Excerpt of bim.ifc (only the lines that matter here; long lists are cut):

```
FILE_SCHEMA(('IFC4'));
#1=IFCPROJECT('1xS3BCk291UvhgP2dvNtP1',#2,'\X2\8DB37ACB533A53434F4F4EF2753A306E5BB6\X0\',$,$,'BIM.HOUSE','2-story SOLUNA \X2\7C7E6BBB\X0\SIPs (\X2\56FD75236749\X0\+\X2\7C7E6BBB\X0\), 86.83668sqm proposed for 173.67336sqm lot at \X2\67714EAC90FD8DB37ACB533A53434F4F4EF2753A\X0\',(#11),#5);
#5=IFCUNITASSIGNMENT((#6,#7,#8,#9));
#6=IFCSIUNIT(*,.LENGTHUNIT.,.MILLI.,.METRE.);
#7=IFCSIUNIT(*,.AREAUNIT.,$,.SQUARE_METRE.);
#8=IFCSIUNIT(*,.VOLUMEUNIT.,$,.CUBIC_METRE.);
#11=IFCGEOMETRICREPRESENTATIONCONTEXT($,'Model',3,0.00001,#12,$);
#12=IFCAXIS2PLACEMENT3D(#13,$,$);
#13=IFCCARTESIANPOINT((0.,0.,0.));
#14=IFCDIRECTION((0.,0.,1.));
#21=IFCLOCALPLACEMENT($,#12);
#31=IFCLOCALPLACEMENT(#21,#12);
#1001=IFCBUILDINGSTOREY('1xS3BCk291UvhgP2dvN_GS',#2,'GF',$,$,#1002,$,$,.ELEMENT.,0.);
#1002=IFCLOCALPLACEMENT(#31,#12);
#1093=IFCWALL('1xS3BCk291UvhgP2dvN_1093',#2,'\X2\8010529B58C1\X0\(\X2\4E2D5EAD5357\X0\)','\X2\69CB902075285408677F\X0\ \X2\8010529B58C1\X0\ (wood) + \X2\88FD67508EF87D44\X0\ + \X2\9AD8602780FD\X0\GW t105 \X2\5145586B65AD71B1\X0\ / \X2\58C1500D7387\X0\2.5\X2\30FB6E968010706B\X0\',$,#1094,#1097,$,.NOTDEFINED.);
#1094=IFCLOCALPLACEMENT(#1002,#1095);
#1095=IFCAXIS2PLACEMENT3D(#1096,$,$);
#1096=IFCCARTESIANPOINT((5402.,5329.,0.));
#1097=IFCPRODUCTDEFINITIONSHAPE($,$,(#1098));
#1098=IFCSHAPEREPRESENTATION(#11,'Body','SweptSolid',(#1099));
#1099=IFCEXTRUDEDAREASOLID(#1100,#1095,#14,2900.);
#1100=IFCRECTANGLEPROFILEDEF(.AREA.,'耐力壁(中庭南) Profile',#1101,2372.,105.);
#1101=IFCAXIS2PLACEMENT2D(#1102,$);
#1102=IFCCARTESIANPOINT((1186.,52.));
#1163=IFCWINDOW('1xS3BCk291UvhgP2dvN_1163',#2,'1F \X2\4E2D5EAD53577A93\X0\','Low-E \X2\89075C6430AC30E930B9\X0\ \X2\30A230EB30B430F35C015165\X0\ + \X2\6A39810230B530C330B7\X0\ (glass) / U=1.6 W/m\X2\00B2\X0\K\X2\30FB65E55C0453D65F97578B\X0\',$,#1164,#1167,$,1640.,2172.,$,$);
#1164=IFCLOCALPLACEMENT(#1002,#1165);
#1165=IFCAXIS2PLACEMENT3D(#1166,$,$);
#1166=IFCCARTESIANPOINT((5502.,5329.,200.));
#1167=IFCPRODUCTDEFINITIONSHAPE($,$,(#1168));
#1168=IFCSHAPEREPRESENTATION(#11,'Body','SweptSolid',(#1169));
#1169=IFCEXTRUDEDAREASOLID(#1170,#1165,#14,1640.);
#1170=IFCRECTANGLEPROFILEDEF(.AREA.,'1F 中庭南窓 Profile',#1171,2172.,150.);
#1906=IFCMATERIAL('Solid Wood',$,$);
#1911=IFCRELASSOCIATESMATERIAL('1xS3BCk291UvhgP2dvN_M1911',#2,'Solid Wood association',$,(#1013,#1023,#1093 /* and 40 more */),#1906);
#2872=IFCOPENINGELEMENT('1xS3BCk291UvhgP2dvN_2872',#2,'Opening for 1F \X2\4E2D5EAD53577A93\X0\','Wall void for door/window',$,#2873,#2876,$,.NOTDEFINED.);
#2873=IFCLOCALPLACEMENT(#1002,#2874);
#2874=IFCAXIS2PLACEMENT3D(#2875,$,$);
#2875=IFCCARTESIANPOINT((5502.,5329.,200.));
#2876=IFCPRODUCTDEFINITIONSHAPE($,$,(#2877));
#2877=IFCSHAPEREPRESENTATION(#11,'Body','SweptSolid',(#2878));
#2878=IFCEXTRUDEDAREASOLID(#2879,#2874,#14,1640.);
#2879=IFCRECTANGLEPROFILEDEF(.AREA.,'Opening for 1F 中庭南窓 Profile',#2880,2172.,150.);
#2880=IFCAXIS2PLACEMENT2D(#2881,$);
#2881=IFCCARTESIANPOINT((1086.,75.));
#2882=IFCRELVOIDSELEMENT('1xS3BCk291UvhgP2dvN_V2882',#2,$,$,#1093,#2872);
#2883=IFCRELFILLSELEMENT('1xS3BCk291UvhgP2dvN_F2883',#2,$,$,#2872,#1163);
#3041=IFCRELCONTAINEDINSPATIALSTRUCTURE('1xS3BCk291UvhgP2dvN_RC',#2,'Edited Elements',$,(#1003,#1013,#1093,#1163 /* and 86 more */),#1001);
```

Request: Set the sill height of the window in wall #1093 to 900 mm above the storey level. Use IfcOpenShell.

```python
import numpy as np
import ifcopenshell
import ifcopenshell.api.geometry
import ifcopenshell.geom
import ifcopenshell.util.element
import ifcopenshell.util.placement
import ifcopenshell.util.shape
import ifcopenshell.util.unit

model = ifcopenshell.open("bim.ifc")
unit_scale = ifcopenshell.util.unit.calculate_unit_scale(model)

window = model.by_guid("1xS3BCk291UvhgP2dvN_1163")
opening = window.FillsVoids[0].RelatingOpeningElement
storey = ifcopenshell.util.element.get_container(window, ifc_class="IfcBuildingStorey")
level = ifcopenshell.util.placement.get_local_placement(storey.ObjectPlacement)[2, 3]

# The opening's origin need not be at the sill, so measure its lowest point.
shape = ifcopenshell.geom.create_shape(ifcopenshell.geom.settings(), opening)
bottom = ifcopenshell.util.shape.get_shape_bottom_elevation(shape, shape.geometry) / unit_scale
dz = level + 900.0 - bottom

shift = np.array([0.0, 0.0, dz])
# The window is not placed relative to its opening, so move both.
for product in (opening, window):
    matrix = ifcopenshell.util.placement.get_local_placement(product.ObjectPlacement)
    matrix[:3, 3] += shift
    ifcopenshell.api.geometry.edit_object_placement(model, product=product, matrix=matrix, is_si=False)

print(f"moved by {dz * unit_scale:+.3f} m")

model.write("bim_updated.ifc")
```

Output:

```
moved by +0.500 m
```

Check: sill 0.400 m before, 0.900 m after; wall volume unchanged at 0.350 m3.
